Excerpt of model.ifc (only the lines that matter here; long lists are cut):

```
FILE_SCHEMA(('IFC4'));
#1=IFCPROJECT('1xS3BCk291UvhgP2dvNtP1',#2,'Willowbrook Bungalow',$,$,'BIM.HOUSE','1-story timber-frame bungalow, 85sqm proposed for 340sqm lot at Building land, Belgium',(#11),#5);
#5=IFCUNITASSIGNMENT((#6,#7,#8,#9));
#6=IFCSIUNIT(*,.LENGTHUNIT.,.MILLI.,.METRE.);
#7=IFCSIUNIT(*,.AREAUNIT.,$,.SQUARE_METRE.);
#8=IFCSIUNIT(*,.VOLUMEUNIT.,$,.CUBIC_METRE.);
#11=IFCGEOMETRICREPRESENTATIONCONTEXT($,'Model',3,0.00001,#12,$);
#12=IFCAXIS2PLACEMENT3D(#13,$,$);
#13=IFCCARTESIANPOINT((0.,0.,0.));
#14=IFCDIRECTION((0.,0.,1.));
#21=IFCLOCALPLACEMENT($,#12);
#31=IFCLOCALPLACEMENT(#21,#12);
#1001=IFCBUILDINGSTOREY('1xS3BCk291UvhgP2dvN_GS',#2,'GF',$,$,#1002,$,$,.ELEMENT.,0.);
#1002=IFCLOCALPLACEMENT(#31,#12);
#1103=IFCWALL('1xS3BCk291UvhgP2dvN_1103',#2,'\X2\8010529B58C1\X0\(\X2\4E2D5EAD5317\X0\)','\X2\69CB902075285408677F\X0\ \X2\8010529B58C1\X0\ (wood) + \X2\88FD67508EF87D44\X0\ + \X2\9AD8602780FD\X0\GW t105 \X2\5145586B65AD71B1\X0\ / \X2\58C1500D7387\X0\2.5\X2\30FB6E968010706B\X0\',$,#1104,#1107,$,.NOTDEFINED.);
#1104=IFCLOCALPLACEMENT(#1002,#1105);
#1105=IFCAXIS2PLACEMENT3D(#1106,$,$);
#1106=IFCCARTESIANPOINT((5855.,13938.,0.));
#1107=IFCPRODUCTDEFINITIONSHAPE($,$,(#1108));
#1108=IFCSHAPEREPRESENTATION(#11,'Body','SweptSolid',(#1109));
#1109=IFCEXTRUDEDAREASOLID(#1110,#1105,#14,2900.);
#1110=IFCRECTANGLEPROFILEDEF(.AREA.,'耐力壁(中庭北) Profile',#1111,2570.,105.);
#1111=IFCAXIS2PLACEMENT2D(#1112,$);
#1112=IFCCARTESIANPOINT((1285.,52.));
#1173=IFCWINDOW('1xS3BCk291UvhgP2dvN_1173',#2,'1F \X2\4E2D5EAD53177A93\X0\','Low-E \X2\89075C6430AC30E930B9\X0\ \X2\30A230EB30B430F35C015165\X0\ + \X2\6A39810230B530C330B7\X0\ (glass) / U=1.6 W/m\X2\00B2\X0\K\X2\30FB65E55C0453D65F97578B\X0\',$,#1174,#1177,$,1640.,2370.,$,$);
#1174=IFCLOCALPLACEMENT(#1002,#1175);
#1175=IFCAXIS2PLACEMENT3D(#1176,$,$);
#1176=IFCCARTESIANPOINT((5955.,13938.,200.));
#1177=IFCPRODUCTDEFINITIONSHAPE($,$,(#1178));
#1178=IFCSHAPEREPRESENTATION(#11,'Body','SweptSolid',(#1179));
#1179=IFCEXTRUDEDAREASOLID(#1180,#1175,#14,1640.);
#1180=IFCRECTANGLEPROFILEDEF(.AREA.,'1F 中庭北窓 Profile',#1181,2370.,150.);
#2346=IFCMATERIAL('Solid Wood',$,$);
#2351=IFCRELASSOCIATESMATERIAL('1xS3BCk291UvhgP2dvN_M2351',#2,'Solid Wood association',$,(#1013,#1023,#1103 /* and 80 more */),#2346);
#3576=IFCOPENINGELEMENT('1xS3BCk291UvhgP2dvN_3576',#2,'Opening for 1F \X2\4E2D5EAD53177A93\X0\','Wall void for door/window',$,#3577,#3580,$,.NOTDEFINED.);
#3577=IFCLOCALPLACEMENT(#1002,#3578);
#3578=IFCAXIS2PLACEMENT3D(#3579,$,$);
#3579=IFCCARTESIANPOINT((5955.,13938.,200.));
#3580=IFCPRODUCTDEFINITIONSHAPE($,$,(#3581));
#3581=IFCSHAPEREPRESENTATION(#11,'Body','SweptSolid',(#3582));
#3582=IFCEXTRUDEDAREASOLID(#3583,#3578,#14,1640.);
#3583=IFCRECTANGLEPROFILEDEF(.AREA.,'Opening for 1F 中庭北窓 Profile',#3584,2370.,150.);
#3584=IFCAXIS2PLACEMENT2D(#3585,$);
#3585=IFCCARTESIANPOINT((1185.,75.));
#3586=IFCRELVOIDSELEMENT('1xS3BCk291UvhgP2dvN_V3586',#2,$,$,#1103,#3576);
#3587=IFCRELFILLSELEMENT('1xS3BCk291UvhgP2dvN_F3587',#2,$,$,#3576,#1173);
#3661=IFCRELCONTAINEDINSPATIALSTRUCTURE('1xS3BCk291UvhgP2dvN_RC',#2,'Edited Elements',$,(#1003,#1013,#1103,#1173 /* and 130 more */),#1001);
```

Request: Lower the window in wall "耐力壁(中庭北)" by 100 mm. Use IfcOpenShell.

```python
import numpy as np
import ifcopenshell
import ifcopenshell.api.geometry
import ifcopenshell.util.placement
import ifcopenshell.util.unit

model = ifcopenshell.open("model.ifc")
unit_scale = ifcopenshell.util.unit.calculate_unit_scale(model)

window = model.by_guid("1xS3BCk291UvhgP2dvN_1173")
opening = window.FillsVoids[0].RelatingOpeningElement
dz = -100.0

shift = np.array([0.0, 0.0, dz])
# The window is not placed relative to its opening, so move both.
for product in (opening, window):
    matrix = ifcopenshell.util.placement.get_local_placement(product.ObjectPlacement)
    matrix[:3, 3] += shift
    ifcopenshell.api.geometry.edit_object_placement(model, product=product, matrix=matrix, is_si=False)

print(f"moved by {dz * unit_scale:+.3f} m")

model.write("model_updated.ifc")
```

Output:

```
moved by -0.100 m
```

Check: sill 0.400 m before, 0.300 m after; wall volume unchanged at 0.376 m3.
